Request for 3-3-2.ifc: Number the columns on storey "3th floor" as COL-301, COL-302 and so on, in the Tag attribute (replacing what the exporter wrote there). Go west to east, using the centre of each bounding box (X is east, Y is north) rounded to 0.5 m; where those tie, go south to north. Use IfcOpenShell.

First a look at what the model holds.

```python
import ifcopenshell
import ifcopenshell.util.element
import ifcopenshell.util.placement

model = ifcopenshell.open("3-3-2.ifc")
print(model.schema)
storey = next(s for s in model.by_type("IfcBuildingStorey") if s.Name == "3th floor")
columns = [e for e in ifcopenshell.util.element.get_decomposition(storey) if e.is_a("IfcColumn")]
for e in sorted(columns, key=lambda e: e.id()):
    origin = ifcopenshell.util.placement.get_local_placement(e.ObjectPlacement)[:3, 3]
    print(e.id(), e.Tag, e.Name, origin.round(2) + 0.0, sep=" | ")
```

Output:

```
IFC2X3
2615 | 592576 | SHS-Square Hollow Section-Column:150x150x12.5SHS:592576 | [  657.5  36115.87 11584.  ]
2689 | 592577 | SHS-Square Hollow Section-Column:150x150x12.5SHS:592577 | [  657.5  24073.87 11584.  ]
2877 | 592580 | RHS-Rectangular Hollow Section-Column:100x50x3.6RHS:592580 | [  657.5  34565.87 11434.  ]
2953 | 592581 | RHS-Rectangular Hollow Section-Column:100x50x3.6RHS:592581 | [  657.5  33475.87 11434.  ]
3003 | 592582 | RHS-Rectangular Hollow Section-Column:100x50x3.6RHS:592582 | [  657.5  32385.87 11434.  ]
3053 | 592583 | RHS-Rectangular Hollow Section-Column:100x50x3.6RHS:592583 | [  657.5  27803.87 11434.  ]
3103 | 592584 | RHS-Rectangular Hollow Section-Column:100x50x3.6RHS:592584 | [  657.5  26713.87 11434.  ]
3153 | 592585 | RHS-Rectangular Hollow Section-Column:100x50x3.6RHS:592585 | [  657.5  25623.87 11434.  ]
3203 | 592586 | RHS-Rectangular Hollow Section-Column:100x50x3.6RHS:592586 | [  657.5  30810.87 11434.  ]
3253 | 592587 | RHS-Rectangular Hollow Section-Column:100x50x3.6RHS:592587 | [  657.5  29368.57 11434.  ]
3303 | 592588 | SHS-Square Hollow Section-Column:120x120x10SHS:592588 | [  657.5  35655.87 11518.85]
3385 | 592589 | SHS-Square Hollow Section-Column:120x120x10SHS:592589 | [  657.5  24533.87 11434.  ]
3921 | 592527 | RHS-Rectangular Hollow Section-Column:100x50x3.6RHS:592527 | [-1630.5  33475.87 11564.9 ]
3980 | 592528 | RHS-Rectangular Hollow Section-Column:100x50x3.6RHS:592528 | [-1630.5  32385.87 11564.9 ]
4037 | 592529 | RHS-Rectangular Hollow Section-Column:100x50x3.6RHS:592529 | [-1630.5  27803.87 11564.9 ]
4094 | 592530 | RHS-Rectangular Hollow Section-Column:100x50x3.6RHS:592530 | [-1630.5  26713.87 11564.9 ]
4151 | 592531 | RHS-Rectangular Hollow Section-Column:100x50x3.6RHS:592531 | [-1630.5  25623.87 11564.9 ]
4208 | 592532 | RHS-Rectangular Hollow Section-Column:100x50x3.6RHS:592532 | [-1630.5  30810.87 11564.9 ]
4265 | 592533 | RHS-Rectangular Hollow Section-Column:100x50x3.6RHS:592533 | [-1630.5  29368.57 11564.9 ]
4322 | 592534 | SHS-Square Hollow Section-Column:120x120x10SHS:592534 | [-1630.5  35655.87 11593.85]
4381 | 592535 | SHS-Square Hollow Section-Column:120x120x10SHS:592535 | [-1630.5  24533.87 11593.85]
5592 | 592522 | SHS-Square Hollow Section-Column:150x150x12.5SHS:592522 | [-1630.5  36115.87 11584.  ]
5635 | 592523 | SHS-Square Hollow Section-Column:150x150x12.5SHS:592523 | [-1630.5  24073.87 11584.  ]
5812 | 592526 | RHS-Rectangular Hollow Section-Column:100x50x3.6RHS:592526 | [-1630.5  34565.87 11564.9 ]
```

```python
import ifcopenshell
import ifcopenshell.geom
import ifcopenshell.util.element
import ifcopenshell.util.shape

model = ifcopenshell.open("3-3-2.ifc")
settings = ifcopenshell.geom.settings()
settings.set("use-world-coords", True)


def centre(element):
    shape = ifcopenshell.geom.create_shape(settings, element)
    return ifcopenshell.util.shape.get_bbox_centroid(shape.geometry)


storey = next(s for s in model.by_type("IfcBuildingStorey") if s.Name == "3th floor")
columns = [e for e in ifcopenshell.util.element.get_decomposition(storey) if e.is_a("IfcColumn")]

# Insertion points can sit at a corner or the storey origin, so sort by the geometry (in metres).
centres = {e: centre(e) for e in columns}
columns.sort(key=lambda e: (round(centres[e][0] / 0.5), centres[e][1]))

for i, e in enumerate(columns, start=1):
    number = f"COL-3{i:02d}"
    e.Tag = number
    print(e.id(), number)

model.write("3-3-2_updated.ifc")
```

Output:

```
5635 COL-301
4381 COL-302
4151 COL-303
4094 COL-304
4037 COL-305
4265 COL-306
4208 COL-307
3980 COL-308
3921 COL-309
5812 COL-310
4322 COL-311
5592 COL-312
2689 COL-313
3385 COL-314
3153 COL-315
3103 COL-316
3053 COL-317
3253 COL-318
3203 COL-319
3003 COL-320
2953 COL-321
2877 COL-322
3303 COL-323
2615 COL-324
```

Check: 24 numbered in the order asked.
